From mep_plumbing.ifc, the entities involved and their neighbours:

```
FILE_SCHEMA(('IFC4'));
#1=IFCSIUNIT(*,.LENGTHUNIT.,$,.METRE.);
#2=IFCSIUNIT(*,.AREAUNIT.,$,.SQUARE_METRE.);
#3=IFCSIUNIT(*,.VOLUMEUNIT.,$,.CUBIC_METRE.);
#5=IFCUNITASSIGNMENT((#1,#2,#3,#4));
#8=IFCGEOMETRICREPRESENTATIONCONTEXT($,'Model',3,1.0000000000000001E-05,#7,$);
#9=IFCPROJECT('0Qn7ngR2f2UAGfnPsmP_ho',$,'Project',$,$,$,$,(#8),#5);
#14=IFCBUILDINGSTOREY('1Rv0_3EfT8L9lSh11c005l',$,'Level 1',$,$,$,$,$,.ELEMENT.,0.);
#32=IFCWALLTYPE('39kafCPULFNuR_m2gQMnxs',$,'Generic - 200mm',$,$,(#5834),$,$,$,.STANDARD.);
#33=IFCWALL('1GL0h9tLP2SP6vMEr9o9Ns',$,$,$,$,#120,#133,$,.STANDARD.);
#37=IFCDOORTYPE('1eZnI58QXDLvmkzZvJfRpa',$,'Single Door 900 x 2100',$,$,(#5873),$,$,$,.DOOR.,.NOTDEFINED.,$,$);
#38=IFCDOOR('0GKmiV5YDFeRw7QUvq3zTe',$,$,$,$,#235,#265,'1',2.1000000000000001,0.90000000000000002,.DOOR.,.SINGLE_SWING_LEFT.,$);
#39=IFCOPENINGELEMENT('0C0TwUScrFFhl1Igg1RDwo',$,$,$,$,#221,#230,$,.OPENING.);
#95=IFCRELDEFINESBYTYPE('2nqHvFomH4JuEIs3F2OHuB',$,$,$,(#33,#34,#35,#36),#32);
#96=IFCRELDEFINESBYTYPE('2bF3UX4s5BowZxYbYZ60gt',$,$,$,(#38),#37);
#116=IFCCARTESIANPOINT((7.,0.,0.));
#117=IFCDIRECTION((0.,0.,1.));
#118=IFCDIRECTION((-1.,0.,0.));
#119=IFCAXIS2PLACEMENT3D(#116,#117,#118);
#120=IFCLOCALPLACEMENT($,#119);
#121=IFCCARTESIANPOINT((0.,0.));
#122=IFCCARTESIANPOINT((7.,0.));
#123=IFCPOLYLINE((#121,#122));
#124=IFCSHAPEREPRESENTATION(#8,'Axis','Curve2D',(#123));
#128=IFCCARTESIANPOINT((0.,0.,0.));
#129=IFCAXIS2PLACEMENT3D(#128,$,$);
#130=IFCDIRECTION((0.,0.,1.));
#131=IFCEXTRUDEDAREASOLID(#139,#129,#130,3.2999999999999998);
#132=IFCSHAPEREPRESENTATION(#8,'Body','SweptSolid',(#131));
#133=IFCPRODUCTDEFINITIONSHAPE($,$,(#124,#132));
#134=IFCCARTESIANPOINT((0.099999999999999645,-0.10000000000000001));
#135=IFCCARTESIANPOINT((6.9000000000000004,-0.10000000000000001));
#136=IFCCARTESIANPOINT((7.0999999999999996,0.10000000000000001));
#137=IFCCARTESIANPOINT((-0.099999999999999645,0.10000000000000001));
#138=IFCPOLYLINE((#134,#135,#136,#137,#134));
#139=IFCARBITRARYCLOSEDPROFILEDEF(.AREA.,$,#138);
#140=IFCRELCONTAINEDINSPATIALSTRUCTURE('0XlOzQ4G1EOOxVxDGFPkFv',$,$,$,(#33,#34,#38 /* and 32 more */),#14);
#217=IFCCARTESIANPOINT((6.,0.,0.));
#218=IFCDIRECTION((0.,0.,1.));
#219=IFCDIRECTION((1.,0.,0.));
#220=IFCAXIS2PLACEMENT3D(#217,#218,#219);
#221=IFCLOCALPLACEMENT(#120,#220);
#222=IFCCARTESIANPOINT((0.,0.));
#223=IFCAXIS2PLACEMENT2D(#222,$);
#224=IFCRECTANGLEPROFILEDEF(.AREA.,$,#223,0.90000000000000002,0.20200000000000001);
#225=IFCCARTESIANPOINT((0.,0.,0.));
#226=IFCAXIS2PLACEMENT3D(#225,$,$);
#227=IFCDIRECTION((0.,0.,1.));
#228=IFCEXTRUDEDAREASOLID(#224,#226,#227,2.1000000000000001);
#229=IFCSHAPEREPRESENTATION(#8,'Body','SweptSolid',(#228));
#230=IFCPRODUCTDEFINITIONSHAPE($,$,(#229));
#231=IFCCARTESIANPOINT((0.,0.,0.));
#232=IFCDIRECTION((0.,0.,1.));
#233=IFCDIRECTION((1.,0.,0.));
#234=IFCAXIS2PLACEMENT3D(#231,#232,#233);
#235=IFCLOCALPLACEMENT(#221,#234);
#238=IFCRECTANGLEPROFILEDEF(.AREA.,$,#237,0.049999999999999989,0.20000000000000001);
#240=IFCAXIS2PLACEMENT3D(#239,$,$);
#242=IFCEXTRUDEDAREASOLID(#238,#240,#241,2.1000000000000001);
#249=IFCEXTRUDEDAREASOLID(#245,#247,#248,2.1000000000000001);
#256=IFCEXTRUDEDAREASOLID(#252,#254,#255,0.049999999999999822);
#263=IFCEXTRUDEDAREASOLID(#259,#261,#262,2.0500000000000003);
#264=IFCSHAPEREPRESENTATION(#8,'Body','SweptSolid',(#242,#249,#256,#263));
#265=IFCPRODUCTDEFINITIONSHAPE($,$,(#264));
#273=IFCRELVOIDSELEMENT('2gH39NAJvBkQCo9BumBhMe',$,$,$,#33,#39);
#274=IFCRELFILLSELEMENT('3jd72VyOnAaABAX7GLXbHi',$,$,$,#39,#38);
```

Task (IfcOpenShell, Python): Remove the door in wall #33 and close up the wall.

```python
import ifcopenshell
import ifcopenshell.api.feature
import ifcopenshell.api.root
import ifcopenshell.geom
import ifcopenshell.util.shape

model = ifcopenshell.open("mep_plumbing.ifc")
settings = ifcopenshell.geom.settings()


def volume(element):
    """Net volume in cubic metres, openings subtracted."""
    shape = ifcopenshell.geom.create_shape(settings, element)
    return ifcopenshell.util.shape.get_volume(shape.geometry)


door = model.by_guid("0GKmiV5YDFeRw7QUvq3zTe")
opening = door.FillsVoids[0].RelatingOpeningElement
wall = opening.VoidsElements[0].RelatingBuildingElement
before = volume(wall)

ifcopenshell.api.root.remove_product(model, product=door)
ifcopenshell.api.feature.remove_feature(model, feature=opening)

after = volume(wall)

print(f"wall volume {before:.3f} -> {after:.3f} m3")

model.write("mep_plumbing_updated.ifc")
```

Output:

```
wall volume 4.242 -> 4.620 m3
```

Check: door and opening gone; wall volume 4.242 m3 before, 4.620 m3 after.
